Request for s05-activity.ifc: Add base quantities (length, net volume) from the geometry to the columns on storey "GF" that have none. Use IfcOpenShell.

First a look at what the model holds.

```python
import ifcopenshell
import ifcopenshell.util.element
import ifcopenshell.util.unit

model = ifcopenshell.open("s05-activity.ifc")
print(model.schema)
for unit_type in ("LENGTHUNIT", "AREAUNIT", "VOLUMEUNIT"):
    print(unit_type, ifcopenshell.util.unit.calculate_unit_scale(model, unit_type))
storey = next(s for s in model.by_type("IfcBuildingStorey") if s.Name == "GF")
columns = [e for e in ifcopenshell.util.element.get_decomposition(storey) if e.is_a("IfcColumn")]
for e in sorted(columns, key=lambda e: e.id()):
    print(e.id(), e.is_a(), e.Name, list(ifcopenshell.util.element.get_psets(e, qtos_only=True)), sep=" | ")
```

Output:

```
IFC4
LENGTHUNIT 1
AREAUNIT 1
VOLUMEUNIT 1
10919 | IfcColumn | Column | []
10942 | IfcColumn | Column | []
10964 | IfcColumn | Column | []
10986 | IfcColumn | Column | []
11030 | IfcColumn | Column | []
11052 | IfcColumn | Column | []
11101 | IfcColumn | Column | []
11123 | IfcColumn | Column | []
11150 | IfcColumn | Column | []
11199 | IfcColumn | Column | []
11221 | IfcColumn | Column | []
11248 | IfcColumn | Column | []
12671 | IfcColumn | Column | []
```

```python
import ifcopenshell
import ifcopenshell.api.pset
import ifcopenshell.geom
import ifcopenshell.util.element
import ifcopenshell.util.shape
import ifcopenshell.util.unit

model = ifcopenshell.open("s05-activity.ifc")
unit_scale = ifcopenshell.util.unit.calculate_unit_scale(model)
volume_scale = ifcopenshell.util.unit.calculate_unit_scale(model, "VOLUMEUNIT")
settings = ifcopenshell.geom.settings()

storey = next(s for s in model.by_type("IfcBuildingStorey") if s.Name == "GF")
columns = [e for e in ifcopenshell.util.element.get_decomposition(storey) if e.is_a("IfcColumn")]

for e in sorted(columns, key=lambda e: e.id()):
    if ifcopenshell.util.element.get_psets(e, qtos_only=True, should_inherit=False):
        continue
    # Geometry comes back in metres, in the element's own axes.
    shape = ifcopenshell.geom.create_shape(settings, e)
    values = {
        "Length": ifcopenshell.util.shape.get_z(shape.geometry) / unit_scale,
        "NetVolume": ifcopenshell.util.shape.get_volume(shape.geometry) / volume_scale,
    }
    qto = ifcopenshell.api.pset.add_qto(model, product=e, name="Qto_ColumnBaseQuantities")
    ifcopenshell.api.pset.edit_qto(model, qto=qto, properties=values)
    print(e.id(), {k: round(v, 3) for k, v in values.items()})

model.write("s05-activity_edited.ifc")
```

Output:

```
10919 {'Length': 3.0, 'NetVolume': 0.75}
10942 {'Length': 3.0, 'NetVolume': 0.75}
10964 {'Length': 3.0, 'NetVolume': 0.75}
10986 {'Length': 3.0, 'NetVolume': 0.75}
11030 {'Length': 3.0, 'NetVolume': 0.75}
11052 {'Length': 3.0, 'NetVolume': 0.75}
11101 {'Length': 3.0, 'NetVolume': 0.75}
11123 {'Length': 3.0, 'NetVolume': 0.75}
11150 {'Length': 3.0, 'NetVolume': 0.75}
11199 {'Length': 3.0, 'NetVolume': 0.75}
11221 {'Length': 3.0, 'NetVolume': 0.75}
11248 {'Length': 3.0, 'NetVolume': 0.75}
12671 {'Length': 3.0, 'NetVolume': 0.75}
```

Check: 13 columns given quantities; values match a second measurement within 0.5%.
